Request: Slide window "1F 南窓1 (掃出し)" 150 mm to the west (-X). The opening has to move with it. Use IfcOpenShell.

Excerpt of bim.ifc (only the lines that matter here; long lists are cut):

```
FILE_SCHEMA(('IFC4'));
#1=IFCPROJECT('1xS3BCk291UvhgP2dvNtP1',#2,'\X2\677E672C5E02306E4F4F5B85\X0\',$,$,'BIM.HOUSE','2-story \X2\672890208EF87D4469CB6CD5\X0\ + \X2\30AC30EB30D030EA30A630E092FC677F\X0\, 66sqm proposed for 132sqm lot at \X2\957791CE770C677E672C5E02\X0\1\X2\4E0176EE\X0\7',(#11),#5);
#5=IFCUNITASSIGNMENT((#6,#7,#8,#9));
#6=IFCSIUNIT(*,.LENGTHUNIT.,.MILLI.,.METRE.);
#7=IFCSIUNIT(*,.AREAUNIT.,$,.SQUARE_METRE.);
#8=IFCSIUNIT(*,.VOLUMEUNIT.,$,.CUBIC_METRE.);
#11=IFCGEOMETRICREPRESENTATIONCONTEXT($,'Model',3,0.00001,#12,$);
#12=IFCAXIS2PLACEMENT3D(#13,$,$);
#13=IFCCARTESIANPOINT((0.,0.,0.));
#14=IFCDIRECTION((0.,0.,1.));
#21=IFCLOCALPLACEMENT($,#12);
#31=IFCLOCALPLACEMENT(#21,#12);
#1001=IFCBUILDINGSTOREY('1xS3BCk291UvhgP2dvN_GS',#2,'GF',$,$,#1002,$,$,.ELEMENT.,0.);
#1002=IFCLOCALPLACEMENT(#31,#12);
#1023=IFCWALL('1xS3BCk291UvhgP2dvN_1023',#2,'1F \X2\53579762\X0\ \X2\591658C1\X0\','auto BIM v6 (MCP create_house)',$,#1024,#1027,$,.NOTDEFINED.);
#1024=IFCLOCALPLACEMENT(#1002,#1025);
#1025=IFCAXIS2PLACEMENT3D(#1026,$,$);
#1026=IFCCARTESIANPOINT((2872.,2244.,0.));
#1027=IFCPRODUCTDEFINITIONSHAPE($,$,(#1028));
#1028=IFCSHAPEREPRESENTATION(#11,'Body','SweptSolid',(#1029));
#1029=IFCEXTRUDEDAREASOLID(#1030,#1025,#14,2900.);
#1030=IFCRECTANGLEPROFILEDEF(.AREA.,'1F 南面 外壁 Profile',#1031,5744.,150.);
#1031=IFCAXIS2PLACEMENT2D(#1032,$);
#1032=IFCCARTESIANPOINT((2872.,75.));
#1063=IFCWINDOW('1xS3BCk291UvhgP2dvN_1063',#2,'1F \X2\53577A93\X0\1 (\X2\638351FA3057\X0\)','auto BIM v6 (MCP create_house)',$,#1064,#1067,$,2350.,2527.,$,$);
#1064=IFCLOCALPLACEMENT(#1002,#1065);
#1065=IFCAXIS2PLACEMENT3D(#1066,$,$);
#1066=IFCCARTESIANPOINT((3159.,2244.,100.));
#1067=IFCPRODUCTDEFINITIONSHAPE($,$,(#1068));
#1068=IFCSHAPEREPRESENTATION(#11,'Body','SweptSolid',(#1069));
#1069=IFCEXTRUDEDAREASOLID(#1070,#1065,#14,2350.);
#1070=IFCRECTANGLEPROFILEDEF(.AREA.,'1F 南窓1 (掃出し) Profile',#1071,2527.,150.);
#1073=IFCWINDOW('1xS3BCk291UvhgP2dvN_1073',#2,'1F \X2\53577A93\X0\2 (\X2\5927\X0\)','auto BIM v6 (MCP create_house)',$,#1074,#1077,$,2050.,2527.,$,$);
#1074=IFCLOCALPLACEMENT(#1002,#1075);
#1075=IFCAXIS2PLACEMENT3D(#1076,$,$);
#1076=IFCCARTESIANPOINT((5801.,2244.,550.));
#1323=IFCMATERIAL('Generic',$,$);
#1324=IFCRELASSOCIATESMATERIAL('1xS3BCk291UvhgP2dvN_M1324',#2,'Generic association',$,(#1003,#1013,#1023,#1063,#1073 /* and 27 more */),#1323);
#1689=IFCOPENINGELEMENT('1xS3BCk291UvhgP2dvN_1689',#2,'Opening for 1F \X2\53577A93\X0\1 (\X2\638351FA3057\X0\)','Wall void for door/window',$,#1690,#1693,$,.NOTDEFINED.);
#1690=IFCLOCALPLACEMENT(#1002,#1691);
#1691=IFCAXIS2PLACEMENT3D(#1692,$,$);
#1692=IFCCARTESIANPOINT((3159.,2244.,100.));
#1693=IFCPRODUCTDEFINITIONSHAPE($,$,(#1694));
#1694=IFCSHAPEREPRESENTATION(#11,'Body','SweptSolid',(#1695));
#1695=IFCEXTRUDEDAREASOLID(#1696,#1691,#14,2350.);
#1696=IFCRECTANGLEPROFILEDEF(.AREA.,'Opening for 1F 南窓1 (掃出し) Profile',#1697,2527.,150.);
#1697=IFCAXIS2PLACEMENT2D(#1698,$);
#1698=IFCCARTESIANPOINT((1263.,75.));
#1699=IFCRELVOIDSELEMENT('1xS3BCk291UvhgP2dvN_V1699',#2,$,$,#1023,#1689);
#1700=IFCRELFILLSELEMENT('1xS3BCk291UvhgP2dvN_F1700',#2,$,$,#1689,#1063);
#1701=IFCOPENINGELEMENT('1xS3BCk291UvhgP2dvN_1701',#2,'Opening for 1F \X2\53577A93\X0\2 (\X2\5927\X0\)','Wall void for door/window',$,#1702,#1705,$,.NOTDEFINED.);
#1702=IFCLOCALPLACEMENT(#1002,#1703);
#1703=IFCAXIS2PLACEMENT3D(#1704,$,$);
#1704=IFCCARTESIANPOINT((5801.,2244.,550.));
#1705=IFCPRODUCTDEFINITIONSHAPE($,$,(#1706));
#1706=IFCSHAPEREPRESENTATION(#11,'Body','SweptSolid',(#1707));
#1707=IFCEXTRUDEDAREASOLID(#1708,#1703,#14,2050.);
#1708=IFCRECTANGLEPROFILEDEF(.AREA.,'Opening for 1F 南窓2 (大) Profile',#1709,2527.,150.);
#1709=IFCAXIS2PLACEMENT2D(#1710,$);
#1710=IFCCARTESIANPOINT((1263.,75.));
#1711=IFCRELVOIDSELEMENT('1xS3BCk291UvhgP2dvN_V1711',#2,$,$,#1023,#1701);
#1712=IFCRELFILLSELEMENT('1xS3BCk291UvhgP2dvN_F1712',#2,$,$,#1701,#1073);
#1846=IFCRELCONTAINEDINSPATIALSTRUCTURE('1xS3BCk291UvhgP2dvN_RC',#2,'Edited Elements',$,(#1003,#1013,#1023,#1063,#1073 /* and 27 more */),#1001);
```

```python
import ifcopenshell
import ifcopenshell.api.geometry
import ifcopenshell.util.placement
import ifcopenshell.util.unit

model = ifcopenshell.open("bim.ifc")
unit_scale = ifcopenshell.util.unit.calculate_unit_scale(model)

window = model.by_id(1063)
opening = window.FillsVoids[0].RelatingOpeningElement
wall = opening.VoidsElements[0].RelatingBuildingElement

wall_matrix = ifcopenshell.util.placement.get_local_placement(wall.ObjectPlacement)
shift = wall_matrix[:3, 0] * -0.15 / unit_scale
before = ifcopenshell.util.placement.get_local_placement(window.ObjectPlacement)[:3, 3].copy()

# The window is not placed relative to its opening, so move both.
for product in (opening, window):
    matrix = ifcopenshell.util.placement.get_local_placement(product.ObjectPlacement)
    matrix[:3, 3] += shift
    ifcopenshell.api.geometry.edit_object_placement(model, product=product, matrix=matrix, is_si=False)

after = ifcopenshell.util.placement.get_local_placement(window.ObjectPlacement)[:3, 3]
print("window moved by", (after - before).round(3) + 0.0)

model.write("bim_edited.ifc")
```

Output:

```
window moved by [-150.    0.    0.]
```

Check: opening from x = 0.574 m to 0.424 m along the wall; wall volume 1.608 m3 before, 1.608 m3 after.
